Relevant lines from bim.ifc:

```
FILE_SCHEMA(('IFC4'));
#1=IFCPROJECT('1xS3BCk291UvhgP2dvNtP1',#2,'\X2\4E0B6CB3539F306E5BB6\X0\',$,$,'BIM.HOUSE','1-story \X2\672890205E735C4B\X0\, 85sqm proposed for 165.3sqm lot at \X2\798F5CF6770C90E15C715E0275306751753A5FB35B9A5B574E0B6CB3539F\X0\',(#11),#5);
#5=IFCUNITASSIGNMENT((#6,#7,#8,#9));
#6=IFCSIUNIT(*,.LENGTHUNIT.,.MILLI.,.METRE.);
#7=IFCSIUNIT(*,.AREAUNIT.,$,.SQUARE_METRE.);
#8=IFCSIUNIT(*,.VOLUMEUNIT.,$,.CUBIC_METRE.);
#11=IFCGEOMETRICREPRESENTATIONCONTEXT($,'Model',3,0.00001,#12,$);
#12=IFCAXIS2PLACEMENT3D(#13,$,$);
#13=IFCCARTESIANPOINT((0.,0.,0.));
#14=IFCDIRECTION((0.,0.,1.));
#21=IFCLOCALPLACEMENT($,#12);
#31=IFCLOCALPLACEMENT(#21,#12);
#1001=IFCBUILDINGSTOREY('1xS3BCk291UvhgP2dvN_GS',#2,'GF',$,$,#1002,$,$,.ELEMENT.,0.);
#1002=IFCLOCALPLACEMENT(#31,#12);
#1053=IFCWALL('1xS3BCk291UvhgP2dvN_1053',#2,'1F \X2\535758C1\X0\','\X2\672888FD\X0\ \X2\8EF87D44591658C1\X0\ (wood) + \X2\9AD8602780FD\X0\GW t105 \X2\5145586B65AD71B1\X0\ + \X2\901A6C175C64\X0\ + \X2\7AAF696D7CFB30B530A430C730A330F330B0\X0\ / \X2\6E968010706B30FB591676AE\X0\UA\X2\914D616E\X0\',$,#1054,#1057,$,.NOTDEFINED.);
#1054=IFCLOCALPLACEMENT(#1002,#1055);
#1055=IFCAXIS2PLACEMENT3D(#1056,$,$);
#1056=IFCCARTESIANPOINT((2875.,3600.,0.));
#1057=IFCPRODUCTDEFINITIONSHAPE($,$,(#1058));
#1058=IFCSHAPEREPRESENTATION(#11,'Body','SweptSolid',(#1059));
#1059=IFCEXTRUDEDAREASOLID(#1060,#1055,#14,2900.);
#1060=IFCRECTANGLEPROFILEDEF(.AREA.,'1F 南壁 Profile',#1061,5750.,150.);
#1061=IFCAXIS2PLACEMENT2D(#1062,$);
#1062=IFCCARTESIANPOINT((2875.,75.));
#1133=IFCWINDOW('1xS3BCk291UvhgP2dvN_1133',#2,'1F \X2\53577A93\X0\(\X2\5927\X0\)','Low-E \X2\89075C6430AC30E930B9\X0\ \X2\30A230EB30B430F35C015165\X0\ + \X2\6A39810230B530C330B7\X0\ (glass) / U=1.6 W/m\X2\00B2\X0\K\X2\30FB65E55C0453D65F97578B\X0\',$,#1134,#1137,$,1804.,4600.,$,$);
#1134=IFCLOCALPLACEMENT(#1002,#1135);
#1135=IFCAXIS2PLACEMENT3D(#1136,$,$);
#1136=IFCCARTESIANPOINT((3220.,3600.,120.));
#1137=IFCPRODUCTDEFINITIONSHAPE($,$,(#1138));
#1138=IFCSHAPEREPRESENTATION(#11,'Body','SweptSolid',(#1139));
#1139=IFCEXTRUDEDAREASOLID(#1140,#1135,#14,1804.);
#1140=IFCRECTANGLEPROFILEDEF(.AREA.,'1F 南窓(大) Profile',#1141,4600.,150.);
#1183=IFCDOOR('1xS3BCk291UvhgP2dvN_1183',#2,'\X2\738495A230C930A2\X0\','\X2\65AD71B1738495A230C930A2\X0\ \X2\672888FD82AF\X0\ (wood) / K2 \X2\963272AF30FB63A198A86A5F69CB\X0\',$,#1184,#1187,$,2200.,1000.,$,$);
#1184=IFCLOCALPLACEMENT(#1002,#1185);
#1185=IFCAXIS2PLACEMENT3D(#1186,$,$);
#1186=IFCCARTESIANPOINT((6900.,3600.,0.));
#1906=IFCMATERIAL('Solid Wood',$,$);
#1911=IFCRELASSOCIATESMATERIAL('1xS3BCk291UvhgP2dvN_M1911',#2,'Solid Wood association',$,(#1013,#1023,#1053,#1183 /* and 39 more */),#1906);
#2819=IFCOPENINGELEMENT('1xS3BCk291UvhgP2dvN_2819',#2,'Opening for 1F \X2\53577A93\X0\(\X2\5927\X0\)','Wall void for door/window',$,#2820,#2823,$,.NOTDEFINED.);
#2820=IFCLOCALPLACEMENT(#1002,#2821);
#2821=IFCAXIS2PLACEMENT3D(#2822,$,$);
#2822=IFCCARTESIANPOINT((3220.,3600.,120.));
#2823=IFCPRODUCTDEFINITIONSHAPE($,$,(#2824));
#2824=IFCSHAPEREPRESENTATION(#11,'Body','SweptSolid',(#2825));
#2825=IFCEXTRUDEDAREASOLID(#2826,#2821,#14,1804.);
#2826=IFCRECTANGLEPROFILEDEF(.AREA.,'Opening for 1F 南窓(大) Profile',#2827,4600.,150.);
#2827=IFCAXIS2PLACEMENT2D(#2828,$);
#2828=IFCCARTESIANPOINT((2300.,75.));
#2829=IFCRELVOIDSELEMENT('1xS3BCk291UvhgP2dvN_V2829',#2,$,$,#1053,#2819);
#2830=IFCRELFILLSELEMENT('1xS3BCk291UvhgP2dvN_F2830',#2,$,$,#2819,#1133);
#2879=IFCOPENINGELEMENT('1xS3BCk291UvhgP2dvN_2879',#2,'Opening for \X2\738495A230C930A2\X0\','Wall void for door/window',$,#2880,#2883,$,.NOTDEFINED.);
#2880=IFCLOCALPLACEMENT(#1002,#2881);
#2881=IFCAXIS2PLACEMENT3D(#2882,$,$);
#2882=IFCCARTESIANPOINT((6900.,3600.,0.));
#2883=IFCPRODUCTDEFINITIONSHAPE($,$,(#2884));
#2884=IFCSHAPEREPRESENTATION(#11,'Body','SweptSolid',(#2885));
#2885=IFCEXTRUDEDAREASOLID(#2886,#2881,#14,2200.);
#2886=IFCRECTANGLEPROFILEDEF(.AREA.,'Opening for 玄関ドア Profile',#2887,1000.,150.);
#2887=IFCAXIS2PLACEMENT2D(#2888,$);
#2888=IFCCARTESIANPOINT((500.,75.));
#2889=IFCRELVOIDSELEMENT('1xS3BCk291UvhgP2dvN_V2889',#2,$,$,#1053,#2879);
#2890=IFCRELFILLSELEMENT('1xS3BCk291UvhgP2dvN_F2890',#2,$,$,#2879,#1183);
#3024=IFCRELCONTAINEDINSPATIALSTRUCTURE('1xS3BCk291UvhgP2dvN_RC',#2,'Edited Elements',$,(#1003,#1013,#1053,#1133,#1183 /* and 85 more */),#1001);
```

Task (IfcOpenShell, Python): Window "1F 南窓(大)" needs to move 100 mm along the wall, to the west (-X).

```python
import ifcopenshell
import ifcopenshell.api.geometry
import ifcopenshell.util.placement
import ifcopenshell.util.unit

model = ifcopenshell.open("bim.ifc")
unit_scale = ifcopenshell.util.unit.calculate_unit_scale(model)

window = model.by_guid("1xS3BCk291UvhgP2dvN_1133")
opening = window.FillsVoids[0].RelatingOpeningElement
wall = opening.VoidsElements[0].RelatingBuildingElement

wall_matrix = ifcopenshell.util.placement.get_local_placement(wall.ObjectPlacement)
shift = wall_matrix[:3, 0] * -0.1 / unit_scale
before = ifcopenshell.util.placement.get_local_placement(window.ObjectPlacement)[:3, 3].copy()

# The window is not placed relative to its opening, so move both.
for product in (opening, window):
    matrix = ifcopenshell.util.placement.get_local_placement(product.ObjectPlacement)
    matrix[:3, 3] += shift
    ifcopenshell.api.geometry.edit_object_placement(model, product=product, matrix=matrix, is_si=False)

after = ifcopenshell.util.placement.get_local_placement(window.ObjectPlacement)[:3, 3]
print("window moved by", (after - before).round(3) + 0.0)

model.write("bim_updated.ifc")
```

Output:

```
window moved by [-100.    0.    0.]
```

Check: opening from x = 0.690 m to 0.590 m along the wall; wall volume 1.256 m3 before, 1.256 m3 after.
